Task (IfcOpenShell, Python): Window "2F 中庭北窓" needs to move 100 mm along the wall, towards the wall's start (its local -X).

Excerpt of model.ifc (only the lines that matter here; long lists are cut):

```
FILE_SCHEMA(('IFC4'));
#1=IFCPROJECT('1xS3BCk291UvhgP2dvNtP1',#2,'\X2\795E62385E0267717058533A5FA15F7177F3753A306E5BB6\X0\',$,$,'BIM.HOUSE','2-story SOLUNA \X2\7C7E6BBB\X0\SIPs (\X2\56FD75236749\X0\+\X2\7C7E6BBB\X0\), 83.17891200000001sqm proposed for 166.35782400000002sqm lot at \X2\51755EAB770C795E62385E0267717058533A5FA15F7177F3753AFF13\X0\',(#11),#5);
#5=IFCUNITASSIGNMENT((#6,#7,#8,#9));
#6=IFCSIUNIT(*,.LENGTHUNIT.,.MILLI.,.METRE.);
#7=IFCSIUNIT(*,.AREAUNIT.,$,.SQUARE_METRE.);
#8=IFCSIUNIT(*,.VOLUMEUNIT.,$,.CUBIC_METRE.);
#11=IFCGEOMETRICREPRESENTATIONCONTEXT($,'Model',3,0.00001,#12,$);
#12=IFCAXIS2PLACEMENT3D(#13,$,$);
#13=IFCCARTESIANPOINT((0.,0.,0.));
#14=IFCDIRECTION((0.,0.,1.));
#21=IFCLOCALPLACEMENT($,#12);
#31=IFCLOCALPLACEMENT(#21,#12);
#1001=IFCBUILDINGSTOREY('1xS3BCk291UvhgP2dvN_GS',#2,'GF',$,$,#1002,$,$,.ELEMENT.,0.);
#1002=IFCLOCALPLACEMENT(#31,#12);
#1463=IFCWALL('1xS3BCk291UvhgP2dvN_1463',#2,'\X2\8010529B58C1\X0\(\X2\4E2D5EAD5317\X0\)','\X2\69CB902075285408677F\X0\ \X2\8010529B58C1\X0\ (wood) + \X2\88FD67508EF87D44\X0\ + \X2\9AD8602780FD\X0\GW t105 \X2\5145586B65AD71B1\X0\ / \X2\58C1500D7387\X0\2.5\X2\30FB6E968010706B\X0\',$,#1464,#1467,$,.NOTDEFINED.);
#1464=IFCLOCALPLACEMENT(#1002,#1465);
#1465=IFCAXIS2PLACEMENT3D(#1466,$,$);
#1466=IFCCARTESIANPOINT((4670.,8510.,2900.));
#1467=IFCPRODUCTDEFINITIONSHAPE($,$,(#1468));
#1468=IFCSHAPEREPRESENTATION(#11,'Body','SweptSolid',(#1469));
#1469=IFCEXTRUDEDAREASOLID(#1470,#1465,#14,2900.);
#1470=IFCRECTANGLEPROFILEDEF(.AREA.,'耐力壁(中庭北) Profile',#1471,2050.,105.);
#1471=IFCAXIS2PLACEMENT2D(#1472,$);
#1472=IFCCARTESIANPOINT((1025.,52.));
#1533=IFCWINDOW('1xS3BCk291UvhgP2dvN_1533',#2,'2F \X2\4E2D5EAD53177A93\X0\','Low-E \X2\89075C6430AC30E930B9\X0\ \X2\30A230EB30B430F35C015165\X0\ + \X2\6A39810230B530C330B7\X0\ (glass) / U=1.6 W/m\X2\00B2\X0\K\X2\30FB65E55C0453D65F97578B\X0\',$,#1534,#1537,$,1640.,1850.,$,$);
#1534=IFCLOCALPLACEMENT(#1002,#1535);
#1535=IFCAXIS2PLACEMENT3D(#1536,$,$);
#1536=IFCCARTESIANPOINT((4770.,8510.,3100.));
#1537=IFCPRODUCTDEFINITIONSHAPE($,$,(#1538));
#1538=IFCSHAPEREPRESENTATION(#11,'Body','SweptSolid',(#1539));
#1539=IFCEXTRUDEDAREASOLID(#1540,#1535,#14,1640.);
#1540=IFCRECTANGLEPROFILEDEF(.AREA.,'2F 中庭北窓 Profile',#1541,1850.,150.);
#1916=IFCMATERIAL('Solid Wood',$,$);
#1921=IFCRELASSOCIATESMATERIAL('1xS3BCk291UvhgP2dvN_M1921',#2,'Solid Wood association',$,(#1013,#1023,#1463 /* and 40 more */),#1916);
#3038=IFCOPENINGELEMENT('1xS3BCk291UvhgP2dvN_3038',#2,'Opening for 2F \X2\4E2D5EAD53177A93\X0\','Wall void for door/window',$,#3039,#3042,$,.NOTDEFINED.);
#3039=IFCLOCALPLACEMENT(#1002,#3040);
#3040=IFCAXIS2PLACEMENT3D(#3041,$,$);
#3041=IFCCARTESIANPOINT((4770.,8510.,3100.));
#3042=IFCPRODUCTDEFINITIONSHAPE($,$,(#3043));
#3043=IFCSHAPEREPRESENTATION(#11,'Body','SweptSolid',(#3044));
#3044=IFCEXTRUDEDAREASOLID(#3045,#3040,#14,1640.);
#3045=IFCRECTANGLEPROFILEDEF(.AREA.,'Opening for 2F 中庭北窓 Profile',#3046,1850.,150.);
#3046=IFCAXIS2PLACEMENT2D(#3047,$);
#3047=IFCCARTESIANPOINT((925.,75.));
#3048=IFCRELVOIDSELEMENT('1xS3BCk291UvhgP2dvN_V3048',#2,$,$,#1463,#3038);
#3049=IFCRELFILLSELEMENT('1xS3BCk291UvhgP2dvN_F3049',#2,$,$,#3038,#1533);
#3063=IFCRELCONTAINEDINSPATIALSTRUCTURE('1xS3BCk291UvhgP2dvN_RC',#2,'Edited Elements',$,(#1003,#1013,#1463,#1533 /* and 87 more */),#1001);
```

```python
import ifcopenshell
import ifcopenshell.api.geometry
import ifcopenshell.util.placement
import ifcopenshell.util.unit

model = ifcopenshell.open("model.ifc")
unit_scale = ifcopenshell.util.unit.calculate_unit_scale(model)

window = model.by_guid("1xS3BCk291UvhgP2dvN_1533")
opening = window.FillsVoids[0].RelatingOpeningElement
wall = opening.VoidsElements[0].RelatingBuildingElement

wall_matrix = ifcopenshell.util.placement.get_local_placement(wall.ObjectPlacement)
shift = wall_matrix[:3, 0] * -0.1 / unit_scale
before = ifcopenshell.util.placement.get_local_placement(window.ObjectPlacement)[:3, 3].copy()

# The window is not placed relative to its opening, so move both.
for product in (opening, window):
    matrix = ifcopenshell.util.placement.get_local_placement(product.ObjectPlacement)
    matrix[:3, 3] += shift
    ifcopenshell.api.geometry.edit_object_placement(model, product=product, matrix=matrix, is_si=False)

after = ifcopenshell.util.placement.get_local_placement(window.ObjectPlacement)[:3, 3]
print("window moved by", (after - before).round(3) + 0.0)

model.write("model_edited.ifc")
```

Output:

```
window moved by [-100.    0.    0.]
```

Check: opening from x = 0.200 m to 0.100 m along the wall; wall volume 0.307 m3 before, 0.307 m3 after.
